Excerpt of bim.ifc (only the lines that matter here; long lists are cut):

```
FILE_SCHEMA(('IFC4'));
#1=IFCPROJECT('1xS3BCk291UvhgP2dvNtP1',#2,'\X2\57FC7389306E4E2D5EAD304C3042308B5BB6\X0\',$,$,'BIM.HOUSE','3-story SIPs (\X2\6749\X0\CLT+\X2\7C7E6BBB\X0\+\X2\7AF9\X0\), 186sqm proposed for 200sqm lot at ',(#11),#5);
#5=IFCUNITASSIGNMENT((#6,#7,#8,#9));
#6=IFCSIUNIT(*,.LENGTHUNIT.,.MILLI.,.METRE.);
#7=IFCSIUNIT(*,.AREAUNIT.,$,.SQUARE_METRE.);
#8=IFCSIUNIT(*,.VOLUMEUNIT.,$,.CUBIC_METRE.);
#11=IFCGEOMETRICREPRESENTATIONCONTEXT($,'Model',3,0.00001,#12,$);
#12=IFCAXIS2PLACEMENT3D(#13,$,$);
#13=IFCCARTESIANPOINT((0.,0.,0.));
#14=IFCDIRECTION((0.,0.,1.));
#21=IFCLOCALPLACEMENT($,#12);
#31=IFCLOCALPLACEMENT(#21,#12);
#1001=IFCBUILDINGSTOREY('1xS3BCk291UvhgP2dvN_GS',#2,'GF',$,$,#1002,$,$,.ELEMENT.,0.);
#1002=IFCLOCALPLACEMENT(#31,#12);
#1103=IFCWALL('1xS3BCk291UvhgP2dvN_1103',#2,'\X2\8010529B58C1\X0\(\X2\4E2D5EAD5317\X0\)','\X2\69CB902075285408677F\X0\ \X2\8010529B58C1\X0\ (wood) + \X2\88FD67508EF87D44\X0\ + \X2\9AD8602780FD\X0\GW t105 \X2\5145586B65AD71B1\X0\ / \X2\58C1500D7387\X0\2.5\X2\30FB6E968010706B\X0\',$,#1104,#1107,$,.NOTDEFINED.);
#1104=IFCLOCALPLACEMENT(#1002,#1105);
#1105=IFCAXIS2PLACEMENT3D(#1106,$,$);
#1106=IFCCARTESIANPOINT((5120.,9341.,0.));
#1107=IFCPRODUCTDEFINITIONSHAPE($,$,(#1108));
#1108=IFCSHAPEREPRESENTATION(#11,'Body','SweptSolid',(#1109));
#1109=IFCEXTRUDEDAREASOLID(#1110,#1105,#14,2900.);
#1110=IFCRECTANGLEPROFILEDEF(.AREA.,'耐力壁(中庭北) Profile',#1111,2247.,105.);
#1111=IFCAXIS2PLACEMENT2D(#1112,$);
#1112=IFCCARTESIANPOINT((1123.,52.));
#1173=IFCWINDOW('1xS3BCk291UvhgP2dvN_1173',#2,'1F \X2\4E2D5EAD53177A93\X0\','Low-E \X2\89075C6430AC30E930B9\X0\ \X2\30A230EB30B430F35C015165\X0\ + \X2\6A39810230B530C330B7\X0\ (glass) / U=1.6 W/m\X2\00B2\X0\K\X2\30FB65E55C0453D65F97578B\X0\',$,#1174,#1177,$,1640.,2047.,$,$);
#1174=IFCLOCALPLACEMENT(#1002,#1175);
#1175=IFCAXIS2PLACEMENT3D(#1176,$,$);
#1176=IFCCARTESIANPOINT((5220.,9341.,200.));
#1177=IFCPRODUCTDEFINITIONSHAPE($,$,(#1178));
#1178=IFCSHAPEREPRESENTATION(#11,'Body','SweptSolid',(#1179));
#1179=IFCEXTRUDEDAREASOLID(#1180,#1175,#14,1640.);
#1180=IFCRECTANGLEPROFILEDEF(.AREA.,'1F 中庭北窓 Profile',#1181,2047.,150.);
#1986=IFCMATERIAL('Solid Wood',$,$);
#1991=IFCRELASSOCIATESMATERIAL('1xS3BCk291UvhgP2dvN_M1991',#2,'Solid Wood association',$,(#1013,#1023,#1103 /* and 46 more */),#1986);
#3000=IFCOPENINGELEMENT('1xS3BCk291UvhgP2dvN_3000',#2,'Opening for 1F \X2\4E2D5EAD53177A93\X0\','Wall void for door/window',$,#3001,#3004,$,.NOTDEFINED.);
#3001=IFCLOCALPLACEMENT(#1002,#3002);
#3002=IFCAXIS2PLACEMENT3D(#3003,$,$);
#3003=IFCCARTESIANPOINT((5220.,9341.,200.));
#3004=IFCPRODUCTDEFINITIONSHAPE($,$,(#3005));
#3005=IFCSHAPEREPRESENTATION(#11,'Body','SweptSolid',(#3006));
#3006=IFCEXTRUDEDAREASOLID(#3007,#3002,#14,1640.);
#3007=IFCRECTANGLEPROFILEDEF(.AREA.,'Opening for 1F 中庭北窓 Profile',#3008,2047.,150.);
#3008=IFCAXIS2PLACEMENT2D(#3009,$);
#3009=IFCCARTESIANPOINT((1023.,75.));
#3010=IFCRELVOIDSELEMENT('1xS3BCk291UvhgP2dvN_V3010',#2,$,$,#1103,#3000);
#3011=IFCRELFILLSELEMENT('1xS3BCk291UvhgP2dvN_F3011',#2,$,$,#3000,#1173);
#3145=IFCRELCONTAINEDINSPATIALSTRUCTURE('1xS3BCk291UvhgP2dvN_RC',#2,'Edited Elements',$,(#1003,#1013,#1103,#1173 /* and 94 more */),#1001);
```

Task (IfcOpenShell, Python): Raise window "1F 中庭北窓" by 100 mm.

```python
import numpy as np
import ifcopenshell
import ifcopenshell.api.geometry
import ifcopenshell.util.placement
import ifcopenshell.util.unit

model = ifcopenshell.open("bim.ifc")
unit_scale = ifcopenshell.util.unit.calculate_unit_scale(model)

window = model.by_guid("1xS3BCk291UvhgP2dvN_1173")
opening = window.FillsVoids[0].RelatingOpeningElement
dz = 100.0

shift = np.array([0.0, 0.0, dz])
# The window is not placed relative to its opening, so move both.
for product in (opening, window):
    matrix = ifcopenshell.util.placement.get_local_placement(product.ObjectPlacement)
    matrix[:3, 3] += shift
    ifcopenshell.api.geometry.edit_object_placement(model, product=product, matrix=matrix, is_si=False)

print(f"moved by {dz * unit_scale:+.3f} m")

model.write("bim_edited.ifc")
```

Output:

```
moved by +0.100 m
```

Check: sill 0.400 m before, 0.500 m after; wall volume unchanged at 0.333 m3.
